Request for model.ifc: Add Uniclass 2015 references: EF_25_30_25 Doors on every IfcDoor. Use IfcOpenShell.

First a look at what the model holds.

```python
import ifcopenshell

model = ifcopenshell.open("model.ifc")
print(model.schema)
print("classifications:", [c.Name for c in model.by_type("IfcClassification")])
for ifc_class in ("IfcDoor", "IfcRoof", "IfcStair", "IfcWall", "IfcWindow"):
    print(ifc_class, len(model.by_type(ifc_class)))
```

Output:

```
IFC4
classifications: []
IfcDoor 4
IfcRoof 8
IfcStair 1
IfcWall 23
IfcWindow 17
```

```python
import ifcopenshell
import ifcopenshell.api.classification

model = ifcopenshell.open("model.ifc")

system = ifcopenshell.api.classification.add_classification(model, classification="Uniclass 2015")

codes = {
    "IfcDoor": ("EF_25_30_25", "Doors"),
}
for ifc_class, (code, name) in codes.items():
    products = model.by_type(ifc_class)
    ifcopenshell.api.classification.add_reference(
        model, products=products, classification=system, identification=code, name=name
    )
    print(code, len(products))

model.write("model_v2.ifc")
```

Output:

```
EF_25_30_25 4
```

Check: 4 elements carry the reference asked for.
